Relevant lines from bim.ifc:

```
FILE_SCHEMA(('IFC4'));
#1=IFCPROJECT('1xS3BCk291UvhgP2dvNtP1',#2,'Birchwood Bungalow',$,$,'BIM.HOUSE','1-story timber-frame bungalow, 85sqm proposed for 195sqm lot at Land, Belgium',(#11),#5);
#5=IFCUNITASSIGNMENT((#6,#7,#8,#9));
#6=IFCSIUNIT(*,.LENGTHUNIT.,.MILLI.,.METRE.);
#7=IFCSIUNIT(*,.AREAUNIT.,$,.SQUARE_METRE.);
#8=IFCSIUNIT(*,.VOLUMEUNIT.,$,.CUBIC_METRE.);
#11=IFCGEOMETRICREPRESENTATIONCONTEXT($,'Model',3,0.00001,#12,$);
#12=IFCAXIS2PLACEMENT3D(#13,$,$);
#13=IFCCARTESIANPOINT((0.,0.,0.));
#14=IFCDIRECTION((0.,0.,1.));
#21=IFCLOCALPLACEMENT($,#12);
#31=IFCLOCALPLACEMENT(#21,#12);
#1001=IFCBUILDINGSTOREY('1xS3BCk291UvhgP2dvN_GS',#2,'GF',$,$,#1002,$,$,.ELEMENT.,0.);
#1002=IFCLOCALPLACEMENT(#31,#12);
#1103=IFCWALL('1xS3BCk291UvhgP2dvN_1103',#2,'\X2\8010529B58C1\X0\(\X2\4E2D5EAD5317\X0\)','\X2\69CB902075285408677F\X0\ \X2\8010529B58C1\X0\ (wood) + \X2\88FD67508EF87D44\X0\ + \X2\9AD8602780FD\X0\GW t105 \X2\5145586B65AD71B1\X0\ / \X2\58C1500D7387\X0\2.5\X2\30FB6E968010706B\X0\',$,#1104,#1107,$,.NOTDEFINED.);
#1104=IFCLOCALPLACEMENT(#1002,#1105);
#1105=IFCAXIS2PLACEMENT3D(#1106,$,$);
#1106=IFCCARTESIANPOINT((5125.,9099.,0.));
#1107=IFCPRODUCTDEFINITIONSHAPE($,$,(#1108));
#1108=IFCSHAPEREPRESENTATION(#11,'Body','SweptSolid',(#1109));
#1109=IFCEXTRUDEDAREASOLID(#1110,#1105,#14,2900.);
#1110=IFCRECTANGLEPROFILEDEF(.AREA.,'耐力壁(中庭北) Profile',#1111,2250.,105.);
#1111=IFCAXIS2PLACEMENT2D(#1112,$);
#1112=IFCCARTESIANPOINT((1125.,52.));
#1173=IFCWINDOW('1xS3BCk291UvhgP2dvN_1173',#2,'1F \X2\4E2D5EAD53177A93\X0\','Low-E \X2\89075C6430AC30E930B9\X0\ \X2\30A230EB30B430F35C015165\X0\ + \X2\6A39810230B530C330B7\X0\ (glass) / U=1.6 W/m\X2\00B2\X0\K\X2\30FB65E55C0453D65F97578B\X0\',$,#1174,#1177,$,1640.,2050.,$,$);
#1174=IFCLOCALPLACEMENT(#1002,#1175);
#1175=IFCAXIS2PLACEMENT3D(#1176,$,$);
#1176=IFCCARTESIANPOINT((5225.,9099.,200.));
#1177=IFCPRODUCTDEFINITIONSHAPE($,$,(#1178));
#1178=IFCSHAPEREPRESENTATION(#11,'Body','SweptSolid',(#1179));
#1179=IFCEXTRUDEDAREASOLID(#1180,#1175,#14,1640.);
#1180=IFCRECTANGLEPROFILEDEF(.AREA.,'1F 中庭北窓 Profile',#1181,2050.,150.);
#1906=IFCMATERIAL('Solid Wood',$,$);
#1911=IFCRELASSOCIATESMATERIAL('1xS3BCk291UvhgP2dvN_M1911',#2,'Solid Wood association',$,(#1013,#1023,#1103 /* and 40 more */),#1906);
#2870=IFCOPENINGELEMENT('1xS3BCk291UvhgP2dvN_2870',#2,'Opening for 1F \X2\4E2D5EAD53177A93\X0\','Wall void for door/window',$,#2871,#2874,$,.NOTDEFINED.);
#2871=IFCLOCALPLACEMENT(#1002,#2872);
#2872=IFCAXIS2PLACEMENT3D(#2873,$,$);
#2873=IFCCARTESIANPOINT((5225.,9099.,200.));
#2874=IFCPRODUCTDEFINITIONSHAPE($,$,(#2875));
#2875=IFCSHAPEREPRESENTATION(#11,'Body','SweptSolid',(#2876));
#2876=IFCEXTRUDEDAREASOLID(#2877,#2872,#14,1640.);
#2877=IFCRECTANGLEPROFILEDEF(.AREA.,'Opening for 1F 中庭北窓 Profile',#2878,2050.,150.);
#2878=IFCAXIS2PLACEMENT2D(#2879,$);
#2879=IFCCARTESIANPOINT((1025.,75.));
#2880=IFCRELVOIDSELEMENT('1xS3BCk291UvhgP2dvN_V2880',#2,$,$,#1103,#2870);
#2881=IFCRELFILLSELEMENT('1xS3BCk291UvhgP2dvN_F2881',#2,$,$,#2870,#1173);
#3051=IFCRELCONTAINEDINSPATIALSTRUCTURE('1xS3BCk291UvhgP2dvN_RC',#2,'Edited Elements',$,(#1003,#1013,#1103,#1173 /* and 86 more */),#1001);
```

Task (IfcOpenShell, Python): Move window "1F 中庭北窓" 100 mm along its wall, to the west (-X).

```python
import ifcopenshell
import ifcopenshell.api.geometry
import ifcopenshell.util.placement
import ifcopenshell.util.unit

model = ifcopenshell.open("bim.ifc")
unit_scale = ifcopenshell.util.unit.calculate_unit_scale(model)

window = model.by_guid("1xS3BCk291UvhgP2dvN_1173")
opening = window.FillsVoids[0].RelatingOpeningElement
wall = opening.VoidsElements[0].RelatingBuildingElement

wall_matrix = ifcopenshell.util.placement.get_local_placement(wall.ObjectPlacement)
shift = wall_matrix[:3, 0] * -0.1 / unit_scale
before = ifcopenshell.util.placement.get_local_placement(window.ObjectPlacement)[:3, 3].copy()

# The window is not placed relative to its opening, so move both.
for product in (opening, window):
    matrix = ifcopenshell.util.placement.get_local_placement(product.ObjectPlacement)
    matrix[:3, 3] += shift
    ifcopenshell.api.geometry.edit_object_placement(model, product=product, matrix=matrix, is_si=False)

after = ifcopenshell.util.placement.get_local_placement(window.ObjectPlacement)[:3, 3]
print("window moved by", (after - before).round(3) + 0.0)

model.write("bim_updated.ifc")
```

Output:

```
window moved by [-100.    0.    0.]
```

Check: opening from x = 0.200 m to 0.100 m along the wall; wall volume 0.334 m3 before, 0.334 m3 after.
